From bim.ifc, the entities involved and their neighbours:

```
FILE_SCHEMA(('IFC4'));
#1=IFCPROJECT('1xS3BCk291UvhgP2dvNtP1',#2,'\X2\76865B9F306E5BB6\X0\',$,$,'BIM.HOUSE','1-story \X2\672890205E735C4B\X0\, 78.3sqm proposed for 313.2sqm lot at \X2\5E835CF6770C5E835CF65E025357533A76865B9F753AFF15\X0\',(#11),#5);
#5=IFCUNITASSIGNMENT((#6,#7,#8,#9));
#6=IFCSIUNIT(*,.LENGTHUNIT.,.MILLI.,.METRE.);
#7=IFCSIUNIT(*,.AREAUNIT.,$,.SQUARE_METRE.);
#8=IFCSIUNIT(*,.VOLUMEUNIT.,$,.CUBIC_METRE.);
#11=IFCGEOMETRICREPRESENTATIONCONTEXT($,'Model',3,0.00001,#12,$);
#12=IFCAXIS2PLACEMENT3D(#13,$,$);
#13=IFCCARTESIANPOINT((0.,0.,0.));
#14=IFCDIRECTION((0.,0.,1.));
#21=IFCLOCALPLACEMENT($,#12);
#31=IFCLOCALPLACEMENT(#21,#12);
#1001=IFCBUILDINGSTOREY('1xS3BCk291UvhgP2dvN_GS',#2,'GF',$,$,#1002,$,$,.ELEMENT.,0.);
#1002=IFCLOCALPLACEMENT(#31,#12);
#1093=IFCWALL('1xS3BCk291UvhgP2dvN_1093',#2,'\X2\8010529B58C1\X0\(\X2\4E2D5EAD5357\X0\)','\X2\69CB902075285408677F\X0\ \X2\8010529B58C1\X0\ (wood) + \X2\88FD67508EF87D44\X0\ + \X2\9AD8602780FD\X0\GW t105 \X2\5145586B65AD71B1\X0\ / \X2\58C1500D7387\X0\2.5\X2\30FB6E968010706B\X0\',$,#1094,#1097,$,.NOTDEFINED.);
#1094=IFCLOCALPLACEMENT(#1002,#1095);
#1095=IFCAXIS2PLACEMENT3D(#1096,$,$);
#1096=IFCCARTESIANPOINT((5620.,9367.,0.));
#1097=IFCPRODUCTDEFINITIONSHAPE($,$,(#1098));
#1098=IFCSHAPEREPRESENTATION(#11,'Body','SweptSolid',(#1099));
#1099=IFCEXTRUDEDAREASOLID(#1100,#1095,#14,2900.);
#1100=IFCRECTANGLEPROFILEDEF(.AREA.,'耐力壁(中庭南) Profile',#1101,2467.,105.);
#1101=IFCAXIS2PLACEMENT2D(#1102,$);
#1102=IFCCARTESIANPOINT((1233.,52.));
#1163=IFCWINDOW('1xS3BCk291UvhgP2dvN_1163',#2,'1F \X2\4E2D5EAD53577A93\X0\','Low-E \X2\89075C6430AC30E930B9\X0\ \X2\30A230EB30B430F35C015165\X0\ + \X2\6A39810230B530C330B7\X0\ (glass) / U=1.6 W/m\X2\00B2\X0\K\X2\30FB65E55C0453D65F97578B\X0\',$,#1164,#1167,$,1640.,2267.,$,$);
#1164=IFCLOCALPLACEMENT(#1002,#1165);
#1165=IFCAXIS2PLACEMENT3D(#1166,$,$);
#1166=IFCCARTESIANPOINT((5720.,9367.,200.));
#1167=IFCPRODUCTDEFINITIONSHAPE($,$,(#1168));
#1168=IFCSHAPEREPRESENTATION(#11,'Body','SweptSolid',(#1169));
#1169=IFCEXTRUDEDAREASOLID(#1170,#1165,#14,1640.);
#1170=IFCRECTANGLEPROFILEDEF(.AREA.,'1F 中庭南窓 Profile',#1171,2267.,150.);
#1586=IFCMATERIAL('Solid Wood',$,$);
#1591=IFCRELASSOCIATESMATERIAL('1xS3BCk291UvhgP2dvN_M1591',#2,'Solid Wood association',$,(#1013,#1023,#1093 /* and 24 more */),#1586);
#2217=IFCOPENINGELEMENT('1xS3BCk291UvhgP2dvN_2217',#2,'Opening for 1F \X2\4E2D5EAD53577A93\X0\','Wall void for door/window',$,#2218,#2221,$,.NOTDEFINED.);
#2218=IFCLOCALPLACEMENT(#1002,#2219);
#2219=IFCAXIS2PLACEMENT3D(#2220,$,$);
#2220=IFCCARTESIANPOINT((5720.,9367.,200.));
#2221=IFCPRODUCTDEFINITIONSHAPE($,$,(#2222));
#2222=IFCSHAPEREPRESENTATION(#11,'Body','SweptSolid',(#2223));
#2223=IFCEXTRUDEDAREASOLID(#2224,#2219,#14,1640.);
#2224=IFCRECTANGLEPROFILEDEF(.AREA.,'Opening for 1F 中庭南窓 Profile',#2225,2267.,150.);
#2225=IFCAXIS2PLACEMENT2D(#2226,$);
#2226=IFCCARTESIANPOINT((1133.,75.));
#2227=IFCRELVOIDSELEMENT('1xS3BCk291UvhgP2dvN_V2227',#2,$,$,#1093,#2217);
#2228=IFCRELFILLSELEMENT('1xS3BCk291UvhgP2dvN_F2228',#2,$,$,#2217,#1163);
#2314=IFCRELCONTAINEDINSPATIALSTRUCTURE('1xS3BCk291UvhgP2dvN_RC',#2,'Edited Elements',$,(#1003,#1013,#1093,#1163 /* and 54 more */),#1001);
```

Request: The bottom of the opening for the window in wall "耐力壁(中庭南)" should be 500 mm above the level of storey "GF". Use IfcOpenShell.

```python
import numpy as np
import ifcopenshell
import ifcopenshell.api.geometry
import ifcopenshell.geom
import ifcopenshell.util.element
import ifcopenshell.util.placement
import ifcopenshell.util.shape
import ifcopenshell.util.unit

model = ifcopenshell.open("bim.ifc")
unit_scale = ifcopenshell.util.unit.calculate_unit_scale(model)

window = model.by_guid("1xS3BCk291UvhgP2dvN_1163")
opening = window.FillsVoids[0].RelatingOpeningElement
storey = ifcopenshell.util.element.get_container(window, ifc_class="IfcBuildingStorey")
level = ifcopenshell.util.placement.get_local_placement(storey.ObjectPlacement)[2, 3]

# The opening's origin need not be at the sill, so measure its lowest point.
shape = ifcopenshell.geom.create_shape(ifcopenshell.geom.settings(), opening)
bottom = ifcopenshell.util.shape.get_shape_bottom_elevation(shape, shape.geometry) / unit_scale
dz = level + 0.5 / unit_scale - bottom

shift = np.array([0.0, 0.0, dz])
# The window is not placed relative to its opening, so move both.
for product in (opening, window):
    matrix = ifcopenshell.util.placement.get_local_placement(product.ObjectPlacement)
    matrix[:3, 3] += shift
    ifcopenshell.api.geometry.edit_object_placement(model, product=product, matrix=matrix, is_si=False)

print(f"moved by {dz * unit_scale:+.3f} m")

model.write("bim_edited.ifc")
```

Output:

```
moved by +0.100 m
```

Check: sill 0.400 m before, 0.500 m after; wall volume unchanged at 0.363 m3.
